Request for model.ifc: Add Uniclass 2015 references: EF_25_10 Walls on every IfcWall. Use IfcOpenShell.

First a look at what the model holds.

```python
import ifcopenshell

model = ifcopenshell.open("model.ifc")
print(model.schema)
print("classifications:", [c.Name for c in model.by_type("IfcClassification")])
for ifc_class in ("IfcDoor", "IfcRoof", "IfcStair", "IfcWall", "IfcWindow"):
    print(ifc_class, len(model.by_type(ifc_class)))
```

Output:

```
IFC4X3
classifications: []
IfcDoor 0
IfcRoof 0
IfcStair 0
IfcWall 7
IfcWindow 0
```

```python
import ifcopenshell
import ifcopenshell.api.classification

model = ifcopenshell.open("model.ifc")

system = ifcopenshell.api.classification.add_classification(model, classification="Uniclass 2015")

codes = {
    "IfcWall": ("EF_25_10", "Walls"),
}
for ifc_class, (code, name) in codes.items():
    products = model.by_type(ifc_class)
    ifcopenshell.api.classification.add_reference(
        model, products=products, classification=system, identification=code, name=name
    )
    print(code, len(products))

model.write("model_rev.ifc")
```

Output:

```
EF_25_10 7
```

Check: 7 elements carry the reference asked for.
